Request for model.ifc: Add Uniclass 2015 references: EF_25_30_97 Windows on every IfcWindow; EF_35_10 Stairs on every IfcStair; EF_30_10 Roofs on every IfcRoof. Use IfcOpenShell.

First a look at what the model holds.

```python
import ifcopenshell

model = ifcopenshell.open("model.ifc")
print(model.schema)
print("classifications:", [c.Name for c in model.by_type("IfcClassification")])
for ifc_class in ("IfcDoor", "IfcRoof", "IfcStair", "IfcWall", "IfcWindow"):
    print(ifc_class, len(model.by_type(ifc_class)))
```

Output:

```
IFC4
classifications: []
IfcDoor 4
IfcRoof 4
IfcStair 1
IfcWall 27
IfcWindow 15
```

```python
import ifcopenshell
import ifcopenshell.api.classification

model = ifcopenshell.open("model.ifc")

system = ifcopenshell.api.classification.add_classification(model, classification="Uniclass 2015")

codes = {
    "IfcWindow": ("EF_25_30_97", "Windows"),
    "IfcStair": ("EF_35_10", "Stairs"),
    "IfcRoof": ("EF_30_10", "Roofs"),
}
for ifc_class, (code, name) in codes.items():
    products = model.by_type(ifc_class)
    ifcopenshell.api.classification.add_reference(
        model, products=products, classification=system, identification=code, name=name
    )
    print(code, len(products))

model.write("model_rev.ifc")
```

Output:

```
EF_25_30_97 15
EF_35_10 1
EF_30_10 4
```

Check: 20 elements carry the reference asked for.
